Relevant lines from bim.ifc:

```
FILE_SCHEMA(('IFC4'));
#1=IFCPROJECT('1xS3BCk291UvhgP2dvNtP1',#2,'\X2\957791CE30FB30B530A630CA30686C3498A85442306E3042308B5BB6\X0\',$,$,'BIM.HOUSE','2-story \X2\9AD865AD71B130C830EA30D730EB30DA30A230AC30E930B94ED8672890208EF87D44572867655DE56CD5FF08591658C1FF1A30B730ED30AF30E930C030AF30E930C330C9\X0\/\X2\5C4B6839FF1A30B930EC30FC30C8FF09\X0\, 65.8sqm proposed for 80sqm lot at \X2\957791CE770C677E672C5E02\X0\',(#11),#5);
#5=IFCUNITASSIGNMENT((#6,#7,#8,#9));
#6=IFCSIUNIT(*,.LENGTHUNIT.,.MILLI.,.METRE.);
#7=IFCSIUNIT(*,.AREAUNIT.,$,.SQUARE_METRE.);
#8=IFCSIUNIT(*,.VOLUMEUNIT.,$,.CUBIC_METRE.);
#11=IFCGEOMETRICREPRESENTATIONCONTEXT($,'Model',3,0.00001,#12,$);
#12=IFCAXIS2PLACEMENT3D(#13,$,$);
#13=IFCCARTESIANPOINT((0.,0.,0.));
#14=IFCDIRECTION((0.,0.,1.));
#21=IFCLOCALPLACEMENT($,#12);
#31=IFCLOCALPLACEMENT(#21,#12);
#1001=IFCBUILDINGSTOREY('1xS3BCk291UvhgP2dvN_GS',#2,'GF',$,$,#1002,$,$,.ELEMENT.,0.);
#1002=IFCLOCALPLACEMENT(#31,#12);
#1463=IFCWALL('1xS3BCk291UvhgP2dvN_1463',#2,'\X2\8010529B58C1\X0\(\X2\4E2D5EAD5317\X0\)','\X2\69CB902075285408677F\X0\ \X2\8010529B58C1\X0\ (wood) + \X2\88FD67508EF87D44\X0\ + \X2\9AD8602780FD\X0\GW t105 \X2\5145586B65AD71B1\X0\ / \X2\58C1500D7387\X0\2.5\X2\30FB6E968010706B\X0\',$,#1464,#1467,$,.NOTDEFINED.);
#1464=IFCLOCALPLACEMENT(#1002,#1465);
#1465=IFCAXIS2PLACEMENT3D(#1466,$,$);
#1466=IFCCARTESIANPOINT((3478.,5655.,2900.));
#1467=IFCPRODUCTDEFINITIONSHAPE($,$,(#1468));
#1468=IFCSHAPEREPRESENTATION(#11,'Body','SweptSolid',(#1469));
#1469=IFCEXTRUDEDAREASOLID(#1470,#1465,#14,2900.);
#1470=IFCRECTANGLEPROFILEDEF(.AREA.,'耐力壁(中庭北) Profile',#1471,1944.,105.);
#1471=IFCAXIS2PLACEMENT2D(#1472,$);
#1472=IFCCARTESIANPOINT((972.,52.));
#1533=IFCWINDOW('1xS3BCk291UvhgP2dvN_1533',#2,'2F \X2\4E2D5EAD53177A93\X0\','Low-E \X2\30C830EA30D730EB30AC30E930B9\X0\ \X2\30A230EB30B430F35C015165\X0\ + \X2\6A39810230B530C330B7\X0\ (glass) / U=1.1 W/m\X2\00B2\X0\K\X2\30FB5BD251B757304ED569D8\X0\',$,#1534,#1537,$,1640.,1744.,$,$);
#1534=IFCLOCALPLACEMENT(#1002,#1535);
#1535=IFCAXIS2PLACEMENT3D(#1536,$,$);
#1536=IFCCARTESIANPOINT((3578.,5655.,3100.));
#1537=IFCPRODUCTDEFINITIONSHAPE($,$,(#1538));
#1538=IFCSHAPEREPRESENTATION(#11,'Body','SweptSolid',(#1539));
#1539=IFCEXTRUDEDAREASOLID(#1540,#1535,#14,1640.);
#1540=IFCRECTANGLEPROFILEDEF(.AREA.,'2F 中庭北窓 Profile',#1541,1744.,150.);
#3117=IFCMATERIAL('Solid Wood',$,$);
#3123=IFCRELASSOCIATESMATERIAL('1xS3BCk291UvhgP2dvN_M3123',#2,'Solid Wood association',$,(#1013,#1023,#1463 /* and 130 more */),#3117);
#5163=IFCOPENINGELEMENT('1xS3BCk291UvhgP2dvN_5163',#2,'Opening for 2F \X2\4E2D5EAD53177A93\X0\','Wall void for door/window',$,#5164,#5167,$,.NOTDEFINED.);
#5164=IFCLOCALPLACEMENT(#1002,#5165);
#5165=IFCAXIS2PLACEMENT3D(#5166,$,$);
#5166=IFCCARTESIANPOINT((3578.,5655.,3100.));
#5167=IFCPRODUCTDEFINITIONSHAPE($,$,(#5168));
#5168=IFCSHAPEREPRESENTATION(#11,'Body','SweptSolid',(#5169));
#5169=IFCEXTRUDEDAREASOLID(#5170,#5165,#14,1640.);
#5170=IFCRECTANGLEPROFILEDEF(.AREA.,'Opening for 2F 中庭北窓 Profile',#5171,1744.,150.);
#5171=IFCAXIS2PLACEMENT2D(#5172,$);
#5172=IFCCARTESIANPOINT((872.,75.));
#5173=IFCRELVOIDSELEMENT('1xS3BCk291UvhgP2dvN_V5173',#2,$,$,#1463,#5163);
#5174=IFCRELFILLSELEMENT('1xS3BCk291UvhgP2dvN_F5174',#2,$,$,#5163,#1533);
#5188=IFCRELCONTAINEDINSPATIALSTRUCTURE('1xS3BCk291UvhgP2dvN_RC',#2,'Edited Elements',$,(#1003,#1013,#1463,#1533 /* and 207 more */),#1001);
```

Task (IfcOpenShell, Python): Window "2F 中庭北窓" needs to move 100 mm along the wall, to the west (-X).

```python
import ifcopenshell
import ifcopenshell.api.geometry
import ifcopenshell.util.placement

model = ifcopenshell.open("bim.ifc")

window = model.by_guid("1xS3BCk291UvhgP2dvN_1533")
opening = window.FillsVoids[0].RelatingOpeningElement
wall = opening.VoidsElements[0].RelatingBuildingElement

wall_matrix = ifcopenshell.util.placement.get_local_placement(wall.ObjectPlacement)
shift = wall_matrix[:3, 0] * -100.0
before = ifcopenshell.util.placement.get_local_placement(window.ObjectPlacement)[:3, 3].copy()

# The window is not placed relative to its opening, so move both.
for product in (opening, window):
    matrix = ifcopenshell.util.placement.get_local_placement(product.ObjectPlacement)
    matrix[:3, 3] += shift
    ifcopenshell.api.geometry.edit_object_placement(model, product=product, matrix=matrix, is_si=False)

after = ifcopenshell.util.placement.get_local_placement(window.ObjectPlacement)[:3, 3]
print("window moved by", (after - before).round(3) + 0.0)

model.write("bim-out.ifc")
```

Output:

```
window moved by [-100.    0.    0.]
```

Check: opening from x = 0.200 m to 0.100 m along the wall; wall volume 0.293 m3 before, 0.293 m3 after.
